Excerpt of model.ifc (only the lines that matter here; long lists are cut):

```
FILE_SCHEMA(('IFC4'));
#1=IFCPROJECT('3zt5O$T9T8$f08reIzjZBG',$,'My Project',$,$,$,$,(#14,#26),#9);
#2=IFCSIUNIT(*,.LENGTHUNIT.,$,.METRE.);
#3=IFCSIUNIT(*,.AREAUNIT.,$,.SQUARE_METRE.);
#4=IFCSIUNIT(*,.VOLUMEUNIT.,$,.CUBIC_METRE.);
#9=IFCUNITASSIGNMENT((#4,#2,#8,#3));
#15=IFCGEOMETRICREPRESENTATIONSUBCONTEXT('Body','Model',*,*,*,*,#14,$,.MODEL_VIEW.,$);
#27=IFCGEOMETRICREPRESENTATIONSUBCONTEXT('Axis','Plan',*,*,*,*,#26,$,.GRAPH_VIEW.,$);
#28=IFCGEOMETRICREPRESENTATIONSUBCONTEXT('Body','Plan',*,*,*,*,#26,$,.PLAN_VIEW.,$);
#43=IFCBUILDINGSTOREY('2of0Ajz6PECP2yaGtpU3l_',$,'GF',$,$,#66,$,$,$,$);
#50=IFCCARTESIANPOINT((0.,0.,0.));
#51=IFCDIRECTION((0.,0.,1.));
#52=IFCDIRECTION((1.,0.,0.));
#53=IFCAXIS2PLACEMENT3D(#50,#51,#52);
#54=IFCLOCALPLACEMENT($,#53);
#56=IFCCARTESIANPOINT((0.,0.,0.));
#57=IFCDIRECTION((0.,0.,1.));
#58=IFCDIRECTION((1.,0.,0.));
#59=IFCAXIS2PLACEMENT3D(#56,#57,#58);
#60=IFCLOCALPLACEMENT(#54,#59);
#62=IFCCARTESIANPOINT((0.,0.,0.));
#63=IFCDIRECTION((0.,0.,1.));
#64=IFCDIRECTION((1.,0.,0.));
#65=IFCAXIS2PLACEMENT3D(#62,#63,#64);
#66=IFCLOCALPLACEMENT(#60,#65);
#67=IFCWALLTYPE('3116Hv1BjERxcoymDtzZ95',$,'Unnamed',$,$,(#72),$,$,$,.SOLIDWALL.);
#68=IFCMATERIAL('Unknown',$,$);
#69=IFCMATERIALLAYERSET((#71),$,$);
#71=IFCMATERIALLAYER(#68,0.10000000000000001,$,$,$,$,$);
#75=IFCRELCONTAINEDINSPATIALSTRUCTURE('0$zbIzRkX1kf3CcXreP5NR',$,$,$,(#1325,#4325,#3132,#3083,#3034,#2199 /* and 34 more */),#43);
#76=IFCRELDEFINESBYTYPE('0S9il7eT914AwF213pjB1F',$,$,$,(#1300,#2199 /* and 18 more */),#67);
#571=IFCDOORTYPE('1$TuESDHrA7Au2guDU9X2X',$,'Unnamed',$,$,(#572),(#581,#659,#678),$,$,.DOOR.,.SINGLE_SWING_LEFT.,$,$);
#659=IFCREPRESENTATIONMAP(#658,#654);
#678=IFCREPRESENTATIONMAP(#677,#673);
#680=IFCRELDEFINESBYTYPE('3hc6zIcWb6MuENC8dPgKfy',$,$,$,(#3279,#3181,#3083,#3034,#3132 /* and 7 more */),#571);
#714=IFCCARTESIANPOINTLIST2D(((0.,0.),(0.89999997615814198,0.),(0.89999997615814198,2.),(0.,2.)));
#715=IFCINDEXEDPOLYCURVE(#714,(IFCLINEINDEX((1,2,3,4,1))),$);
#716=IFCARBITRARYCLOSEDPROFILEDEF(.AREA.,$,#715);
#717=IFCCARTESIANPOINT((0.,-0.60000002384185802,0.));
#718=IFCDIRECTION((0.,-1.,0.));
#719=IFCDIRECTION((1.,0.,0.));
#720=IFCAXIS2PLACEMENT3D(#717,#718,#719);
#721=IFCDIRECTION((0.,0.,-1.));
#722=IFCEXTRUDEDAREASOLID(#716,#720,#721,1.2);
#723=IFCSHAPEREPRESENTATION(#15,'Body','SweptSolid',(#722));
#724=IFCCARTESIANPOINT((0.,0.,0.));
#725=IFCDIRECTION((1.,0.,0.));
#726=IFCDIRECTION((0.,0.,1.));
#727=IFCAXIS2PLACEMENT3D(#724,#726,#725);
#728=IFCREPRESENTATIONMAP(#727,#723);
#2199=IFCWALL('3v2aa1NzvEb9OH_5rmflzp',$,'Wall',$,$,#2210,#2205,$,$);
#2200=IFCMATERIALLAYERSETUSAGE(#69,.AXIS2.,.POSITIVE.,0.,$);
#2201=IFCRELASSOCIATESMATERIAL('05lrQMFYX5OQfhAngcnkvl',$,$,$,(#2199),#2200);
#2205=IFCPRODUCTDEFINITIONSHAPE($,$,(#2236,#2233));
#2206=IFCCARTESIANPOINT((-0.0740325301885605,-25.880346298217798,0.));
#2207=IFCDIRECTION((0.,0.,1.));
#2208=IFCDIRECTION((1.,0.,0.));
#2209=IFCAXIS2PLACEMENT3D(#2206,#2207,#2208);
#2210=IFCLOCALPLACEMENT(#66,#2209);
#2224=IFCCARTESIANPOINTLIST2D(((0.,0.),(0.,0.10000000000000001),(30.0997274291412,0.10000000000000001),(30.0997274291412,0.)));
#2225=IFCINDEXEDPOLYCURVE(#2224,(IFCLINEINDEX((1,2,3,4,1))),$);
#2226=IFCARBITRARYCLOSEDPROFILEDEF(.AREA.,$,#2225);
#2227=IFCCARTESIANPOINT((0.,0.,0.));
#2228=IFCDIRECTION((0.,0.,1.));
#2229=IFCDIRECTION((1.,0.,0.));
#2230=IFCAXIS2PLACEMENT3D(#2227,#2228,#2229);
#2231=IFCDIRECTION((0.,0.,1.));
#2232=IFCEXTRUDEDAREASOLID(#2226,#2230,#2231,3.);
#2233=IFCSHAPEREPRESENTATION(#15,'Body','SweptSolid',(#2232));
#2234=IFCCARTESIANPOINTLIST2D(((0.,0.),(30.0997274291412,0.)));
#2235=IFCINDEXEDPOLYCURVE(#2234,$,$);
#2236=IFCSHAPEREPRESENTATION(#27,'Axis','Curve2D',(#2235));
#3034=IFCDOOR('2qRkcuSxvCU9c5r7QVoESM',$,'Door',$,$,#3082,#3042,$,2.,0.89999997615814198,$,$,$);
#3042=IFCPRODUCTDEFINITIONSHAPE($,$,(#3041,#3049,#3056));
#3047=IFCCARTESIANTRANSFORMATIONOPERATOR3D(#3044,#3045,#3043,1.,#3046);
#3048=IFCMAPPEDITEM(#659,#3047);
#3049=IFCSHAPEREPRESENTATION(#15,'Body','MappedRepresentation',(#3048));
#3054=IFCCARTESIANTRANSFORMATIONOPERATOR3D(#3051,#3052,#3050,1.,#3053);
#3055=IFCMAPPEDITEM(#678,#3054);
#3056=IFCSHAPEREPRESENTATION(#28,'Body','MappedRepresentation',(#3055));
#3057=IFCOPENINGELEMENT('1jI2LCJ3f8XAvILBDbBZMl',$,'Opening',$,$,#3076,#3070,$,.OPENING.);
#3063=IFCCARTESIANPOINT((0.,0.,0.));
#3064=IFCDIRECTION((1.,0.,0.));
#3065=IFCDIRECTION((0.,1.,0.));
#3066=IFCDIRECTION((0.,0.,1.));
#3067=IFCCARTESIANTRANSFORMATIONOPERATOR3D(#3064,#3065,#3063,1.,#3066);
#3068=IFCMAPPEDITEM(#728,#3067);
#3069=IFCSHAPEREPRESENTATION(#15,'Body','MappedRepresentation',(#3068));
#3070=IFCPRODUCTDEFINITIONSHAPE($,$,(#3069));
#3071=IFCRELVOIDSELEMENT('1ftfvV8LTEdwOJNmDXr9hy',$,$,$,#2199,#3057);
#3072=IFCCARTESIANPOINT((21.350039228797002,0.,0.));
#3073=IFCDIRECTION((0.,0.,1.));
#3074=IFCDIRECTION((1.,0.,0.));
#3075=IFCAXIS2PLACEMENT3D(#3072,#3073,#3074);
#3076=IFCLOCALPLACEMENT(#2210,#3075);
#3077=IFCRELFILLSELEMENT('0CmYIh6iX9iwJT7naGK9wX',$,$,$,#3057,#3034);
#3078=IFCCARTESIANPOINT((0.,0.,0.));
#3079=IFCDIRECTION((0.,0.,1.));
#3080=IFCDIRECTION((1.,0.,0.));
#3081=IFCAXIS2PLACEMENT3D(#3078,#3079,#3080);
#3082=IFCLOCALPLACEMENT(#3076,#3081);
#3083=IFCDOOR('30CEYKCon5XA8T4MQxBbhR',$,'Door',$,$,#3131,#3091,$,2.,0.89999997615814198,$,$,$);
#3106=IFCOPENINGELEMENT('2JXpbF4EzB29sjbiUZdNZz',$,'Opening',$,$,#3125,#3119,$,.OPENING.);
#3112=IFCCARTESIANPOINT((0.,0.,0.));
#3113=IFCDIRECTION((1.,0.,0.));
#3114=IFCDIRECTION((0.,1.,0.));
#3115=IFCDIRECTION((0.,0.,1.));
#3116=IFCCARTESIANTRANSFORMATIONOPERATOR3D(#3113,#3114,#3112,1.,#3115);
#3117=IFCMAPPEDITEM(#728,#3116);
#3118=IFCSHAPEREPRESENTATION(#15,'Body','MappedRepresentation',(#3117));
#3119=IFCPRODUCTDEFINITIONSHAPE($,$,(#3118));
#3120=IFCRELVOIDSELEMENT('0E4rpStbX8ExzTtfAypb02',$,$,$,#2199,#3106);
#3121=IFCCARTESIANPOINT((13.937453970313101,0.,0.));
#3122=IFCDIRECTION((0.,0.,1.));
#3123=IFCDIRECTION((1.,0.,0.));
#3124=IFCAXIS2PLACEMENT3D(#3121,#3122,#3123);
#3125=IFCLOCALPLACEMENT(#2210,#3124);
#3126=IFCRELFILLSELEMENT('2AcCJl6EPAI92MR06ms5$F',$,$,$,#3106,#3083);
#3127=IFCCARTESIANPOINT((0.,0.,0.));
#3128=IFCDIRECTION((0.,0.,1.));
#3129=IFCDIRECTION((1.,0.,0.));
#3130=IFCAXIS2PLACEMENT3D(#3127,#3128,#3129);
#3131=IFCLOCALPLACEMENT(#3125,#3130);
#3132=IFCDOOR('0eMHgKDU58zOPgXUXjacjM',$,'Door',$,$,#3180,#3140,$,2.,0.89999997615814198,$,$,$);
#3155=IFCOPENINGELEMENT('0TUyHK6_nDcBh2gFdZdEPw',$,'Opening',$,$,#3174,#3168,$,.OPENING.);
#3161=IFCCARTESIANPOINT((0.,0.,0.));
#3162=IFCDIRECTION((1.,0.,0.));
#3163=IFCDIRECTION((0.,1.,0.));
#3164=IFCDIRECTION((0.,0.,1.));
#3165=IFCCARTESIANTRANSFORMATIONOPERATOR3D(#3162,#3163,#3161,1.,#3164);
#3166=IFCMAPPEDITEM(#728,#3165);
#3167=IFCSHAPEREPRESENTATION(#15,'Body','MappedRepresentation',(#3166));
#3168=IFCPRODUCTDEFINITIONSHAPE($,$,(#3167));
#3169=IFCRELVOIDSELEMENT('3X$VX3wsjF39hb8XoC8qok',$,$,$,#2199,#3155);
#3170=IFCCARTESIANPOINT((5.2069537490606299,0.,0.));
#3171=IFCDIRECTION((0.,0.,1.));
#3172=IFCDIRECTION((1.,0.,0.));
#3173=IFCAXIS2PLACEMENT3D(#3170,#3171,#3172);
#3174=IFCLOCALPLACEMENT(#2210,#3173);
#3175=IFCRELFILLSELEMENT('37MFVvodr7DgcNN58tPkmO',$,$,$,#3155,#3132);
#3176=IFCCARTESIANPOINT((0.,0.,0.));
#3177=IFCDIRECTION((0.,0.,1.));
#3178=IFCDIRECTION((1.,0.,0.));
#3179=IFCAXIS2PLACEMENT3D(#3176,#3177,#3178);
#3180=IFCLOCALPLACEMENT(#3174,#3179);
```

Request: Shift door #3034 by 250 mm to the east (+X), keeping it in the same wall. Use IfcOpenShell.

```python
import ifcopenshell
import ifcopenshell.api.geometry
import ifcopenshell.util.placement

model = ifcopenshell.open("model.ifc")

door = model.by_guid("2qRkcuSxvCU9c5r7QVoESM")
opening = door.FillsVoids[0].RelatingOpeningElement
wall = opening.VoidsElements[0].RelatingBuildingElement

wall_matrix = ifcopenshell.util.placement.get_local_placement(wall.ObjectPlacement)
shift = wall_matrix[:3, 0] * 0.25
before = ifcopenshell.util.placement.get_local_placement(door.ObjectPlacement)[:3, 3].copy()

# The door is placed relative to its opening, so it follows when the opening moves.
matrix = ifcopenshell.util.placement.get_local_placement(opening.ObjectPlacement)
matrix[:3, 3] += shift
ifcopenshell.api.geometry.edit_object_placement(
    model, product=opening, matrix=matrix, is_si=False, should_transform_children=True
)

after = ifcopenshell.util.placement.get_local_placement(door.ObjectPlacement)[:3, 3]
print("door moved by", (after - before).round(3) + 0.0)

model.write("model_v2.ifc")
```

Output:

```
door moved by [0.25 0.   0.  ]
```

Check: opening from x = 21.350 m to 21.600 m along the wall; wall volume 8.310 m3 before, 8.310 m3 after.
